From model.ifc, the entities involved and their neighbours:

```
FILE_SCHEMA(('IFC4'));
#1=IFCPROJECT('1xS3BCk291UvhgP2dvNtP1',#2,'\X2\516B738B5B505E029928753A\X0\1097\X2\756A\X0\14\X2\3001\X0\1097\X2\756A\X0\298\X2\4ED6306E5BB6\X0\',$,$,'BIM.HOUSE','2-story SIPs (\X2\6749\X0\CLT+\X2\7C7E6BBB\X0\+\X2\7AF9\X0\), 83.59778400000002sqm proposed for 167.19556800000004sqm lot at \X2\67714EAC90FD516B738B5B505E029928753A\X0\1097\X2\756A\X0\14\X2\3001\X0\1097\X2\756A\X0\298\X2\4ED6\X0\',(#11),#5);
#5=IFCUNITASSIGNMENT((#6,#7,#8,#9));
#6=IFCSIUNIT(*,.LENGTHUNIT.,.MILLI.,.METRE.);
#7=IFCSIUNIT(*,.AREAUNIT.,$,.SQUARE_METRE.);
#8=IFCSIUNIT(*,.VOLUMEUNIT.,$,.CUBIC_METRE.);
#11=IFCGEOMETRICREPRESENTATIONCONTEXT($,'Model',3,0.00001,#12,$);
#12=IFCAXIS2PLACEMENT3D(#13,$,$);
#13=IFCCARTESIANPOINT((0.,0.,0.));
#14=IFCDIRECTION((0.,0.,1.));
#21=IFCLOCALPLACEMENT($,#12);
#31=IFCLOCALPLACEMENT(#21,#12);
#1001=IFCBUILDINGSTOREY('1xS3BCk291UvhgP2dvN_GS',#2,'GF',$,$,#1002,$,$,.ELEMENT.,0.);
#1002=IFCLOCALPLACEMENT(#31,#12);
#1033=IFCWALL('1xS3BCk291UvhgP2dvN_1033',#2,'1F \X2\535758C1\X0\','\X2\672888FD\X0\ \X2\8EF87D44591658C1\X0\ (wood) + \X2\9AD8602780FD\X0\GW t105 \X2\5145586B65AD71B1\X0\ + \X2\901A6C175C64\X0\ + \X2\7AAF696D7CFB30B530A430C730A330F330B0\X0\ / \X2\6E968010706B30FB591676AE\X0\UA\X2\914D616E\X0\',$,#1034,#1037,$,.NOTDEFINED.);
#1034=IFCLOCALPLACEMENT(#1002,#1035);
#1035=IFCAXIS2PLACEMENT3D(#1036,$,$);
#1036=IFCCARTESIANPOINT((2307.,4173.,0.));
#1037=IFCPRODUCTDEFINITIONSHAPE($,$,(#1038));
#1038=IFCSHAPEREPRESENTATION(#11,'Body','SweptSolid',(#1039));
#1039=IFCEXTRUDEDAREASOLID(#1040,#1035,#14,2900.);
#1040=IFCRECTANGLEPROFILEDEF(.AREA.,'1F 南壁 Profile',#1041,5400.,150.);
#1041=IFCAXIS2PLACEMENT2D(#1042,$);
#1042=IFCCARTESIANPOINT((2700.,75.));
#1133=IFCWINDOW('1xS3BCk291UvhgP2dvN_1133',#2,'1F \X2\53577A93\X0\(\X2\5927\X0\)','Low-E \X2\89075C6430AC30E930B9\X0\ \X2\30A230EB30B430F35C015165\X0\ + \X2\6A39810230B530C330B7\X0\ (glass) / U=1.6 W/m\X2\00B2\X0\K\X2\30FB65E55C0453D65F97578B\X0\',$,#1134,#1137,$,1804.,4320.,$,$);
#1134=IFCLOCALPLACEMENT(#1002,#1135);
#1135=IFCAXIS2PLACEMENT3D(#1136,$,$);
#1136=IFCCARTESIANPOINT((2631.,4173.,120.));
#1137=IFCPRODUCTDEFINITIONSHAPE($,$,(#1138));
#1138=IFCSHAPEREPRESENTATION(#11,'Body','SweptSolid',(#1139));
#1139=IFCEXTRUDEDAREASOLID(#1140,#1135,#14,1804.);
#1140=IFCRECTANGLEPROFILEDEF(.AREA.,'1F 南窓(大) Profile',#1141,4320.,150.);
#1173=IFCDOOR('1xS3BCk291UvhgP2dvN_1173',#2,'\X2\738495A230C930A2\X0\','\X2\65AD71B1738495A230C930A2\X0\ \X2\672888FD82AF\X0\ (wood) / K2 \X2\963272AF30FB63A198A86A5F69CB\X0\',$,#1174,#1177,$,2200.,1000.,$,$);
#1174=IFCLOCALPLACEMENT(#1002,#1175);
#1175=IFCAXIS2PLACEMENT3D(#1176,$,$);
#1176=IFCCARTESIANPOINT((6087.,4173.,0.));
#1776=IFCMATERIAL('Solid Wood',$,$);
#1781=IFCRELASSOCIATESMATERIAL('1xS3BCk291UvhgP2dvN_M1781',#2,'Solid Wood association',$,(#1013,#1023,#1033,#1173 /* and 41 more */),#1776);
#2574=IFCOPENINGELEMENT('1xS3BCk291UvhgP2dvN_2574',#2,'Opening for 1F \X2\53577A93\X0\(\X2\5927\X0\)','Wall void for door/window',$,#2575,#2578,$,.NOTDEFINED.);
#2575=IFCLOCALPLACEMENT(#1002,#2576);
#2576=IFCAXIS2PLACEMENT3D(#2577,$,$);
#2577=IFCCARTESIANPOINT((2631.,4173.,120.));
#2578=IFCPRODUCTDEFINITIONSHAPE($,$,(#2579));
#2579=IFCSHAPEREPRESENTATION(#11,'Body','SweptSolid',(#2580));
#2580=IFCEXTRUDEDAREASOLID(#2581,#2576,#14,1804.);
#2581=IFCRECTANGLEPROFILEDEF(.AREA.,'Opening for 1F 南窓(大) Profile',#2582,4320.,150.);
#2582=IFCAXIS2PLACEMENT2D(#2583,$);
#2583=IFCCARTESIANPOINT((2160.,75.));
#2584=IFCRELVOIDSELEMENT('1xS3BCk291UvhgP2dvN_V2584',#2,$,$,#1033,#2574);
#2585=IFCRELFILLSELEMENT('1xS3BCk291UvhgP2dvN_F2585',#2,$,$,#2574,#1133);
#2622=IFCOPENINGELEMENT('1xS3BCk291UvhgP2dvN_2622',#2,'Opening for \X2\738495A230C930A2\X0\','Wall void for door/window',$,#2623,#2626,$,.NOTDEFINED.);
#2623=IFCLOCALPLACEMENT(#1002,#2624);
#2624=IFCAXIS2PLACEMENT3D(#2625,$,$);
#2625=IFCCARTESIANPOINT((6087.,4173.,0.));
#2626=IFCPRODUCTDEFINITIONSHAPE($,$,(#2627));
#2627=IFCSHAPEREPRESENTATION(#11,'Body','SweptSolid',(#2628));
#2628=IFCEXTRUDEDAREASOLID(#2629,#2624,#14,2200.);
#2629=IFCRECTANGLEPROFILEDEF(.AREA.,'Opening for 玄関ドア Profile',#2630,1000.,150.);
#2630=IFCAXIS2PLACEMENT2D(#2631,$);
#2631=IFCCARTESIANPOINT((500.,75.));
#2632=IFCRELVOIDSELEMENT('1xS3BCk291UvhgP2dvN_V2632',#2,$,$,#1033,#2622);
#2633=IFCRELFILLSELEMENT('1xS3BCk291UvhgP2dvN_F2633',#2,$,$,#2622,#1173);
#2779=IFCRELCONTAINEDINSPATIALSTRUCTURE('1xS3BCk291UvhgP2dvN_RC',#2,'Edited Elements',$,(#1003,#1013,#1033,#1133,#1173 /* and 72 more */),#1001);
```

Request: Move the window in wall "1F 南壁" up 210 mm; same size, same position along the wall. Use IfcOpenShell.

```python
import numpy as np
import ifcopenshell
import ifcopenshell.api.geometry
import ifcopenshell.util.placement
import ifcopenshell.util.unit

model = ifcopenshell.open("model.ifc")
unit_scale = ifcopenshell.util.unit.calculate_unit_scale(model)

window = model.by_id(1133)
opening = window.FillsVoids[0].RelatingOpeningElement
dz = 0.21 / unit_scale

shift = np.array([0.0, 0.0, dz])
# The window is not placed relative to its opening, so move both.
for product in (opening, window):
    matrix = ifcopenshell.util.placement.get_local_placement(product.ObjectPlacement)
    matrix[:3, 3] += shift
    ifcopenshell.api.geometry.edit_object_placement(model, product=product, matrix=matrix, is_si=False)

print(f"moved by {dz * unit_scale:+.3f} m")

model.write("model_updated.ifc")
```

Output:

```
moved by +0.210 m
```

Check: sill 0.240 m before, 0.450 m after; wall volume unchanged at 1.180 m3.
